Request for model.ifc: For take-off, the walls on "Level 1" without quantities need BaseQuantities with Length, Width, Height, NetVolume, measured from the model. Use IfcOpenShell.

First a look at what the model holds.

```python
import ifcopenshell
import ifcopenshell.util.element
import ifcopenshell.util.unit

model = ifcopenshell.open("model.ifc")
print(model.schema)
for unit_type in ("LENGTHUNIT", "AREAUNIT", "VOLUMEUNIT"):
    print(unit_type, ifcopenshell.util.unit.calculate_unit_scale(model, unit_type))
storey = next(s for s in model.by_type("IfcBuildingStorey") if s.Name == "Level 1")
walls = [e for e in ifcopenshell.util.element.get_decomposition(storey) if e.is_a("IfcWall")]
for e in sorted(walls, key=lambda e: e.id()):
    print(e.id(), e.is_a(), e.Name, list(ifcopenshell.util.element.get_psets(e, qtos_only=True)), sep=" | ")
```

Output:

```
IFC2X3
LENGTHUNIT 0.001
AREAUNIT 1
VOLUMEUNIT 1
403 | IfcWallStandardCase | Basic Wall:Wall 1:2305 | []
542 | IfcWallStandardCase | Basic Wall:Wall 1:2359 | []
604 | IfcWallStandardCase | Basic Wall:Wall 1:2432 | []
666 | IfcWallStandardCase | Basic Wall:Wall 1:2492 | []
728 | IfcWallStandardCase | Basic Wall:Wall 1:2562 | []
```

```python
import ifcopenshell
import ifcopenshell.api.pset
import ifcopenshell.geom
import ifcopenshell.util.element
import ifcopenshell.util.shape
import ifcopenshell.util.unit

model = ifcopenshell.open("model.ifc")
unit_scale = ifcopenshell.util.unit.calculate_unit_scale(model)
volume_scale = ifcopenshell.util.unit.calculate_unit_scale(model, "VOLUMEUNIT")
settings = ifcopenshell.geom.settings()

storey = next(s for s in model.by_type("IfcBuildingStorey") if s.Name == "Level 1")
walls = [e for e in ifcopenshell.util.element.get_decomposition(storey) if e.is_a("IfcWall")]

for e in sorted(walls, key=lambda e: e.id()):
    if ifcopenshell.util.element.get_psets(e, qtos_only=True, should_inherit=False):
        continue
    # Geometry comes back in metres, in the element's own axes.
    shape = ifcopenshell.geom.create_shape(settings, e)
    values = {
        "Length": ifcopenshell.util.shape.get_x(shape.geometry) / unit_scale,
        "Width": ifcopenshell.util.shape.get_y(shape.geometry) / unit_scale,
        "Height": ifcopenshell.util.shape.get_z(shape.geometry) / unit_scale,
        "NetVolume": ifcopenshell.util.shape.get_volume(shape.geometry) / volume_scale,
    }
    qto = ifcopenshell.api.pset.add_qto(model, product=e, name="BaseQuantities")
    ifcopenshell.api.pset.edit_qto(model, qto=qto, properties=values)
    print(e.id(), {k: round(v, 3) for k, v in values.items()})

model.write("model_rev.ifc")
```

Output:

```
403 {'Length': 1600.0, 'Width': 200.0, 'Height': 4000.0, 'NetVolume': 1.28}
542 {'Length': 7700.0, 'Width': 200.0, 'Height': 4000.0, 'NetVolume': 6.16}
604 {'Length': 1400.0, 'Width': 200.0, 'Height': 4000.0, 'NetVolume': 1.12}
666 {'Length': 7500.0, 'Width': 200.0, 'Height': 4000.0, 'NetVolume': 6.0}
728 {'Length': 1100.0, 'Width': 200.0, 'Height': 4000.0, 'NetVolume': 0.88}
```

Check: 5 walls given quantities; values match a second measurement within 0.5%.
